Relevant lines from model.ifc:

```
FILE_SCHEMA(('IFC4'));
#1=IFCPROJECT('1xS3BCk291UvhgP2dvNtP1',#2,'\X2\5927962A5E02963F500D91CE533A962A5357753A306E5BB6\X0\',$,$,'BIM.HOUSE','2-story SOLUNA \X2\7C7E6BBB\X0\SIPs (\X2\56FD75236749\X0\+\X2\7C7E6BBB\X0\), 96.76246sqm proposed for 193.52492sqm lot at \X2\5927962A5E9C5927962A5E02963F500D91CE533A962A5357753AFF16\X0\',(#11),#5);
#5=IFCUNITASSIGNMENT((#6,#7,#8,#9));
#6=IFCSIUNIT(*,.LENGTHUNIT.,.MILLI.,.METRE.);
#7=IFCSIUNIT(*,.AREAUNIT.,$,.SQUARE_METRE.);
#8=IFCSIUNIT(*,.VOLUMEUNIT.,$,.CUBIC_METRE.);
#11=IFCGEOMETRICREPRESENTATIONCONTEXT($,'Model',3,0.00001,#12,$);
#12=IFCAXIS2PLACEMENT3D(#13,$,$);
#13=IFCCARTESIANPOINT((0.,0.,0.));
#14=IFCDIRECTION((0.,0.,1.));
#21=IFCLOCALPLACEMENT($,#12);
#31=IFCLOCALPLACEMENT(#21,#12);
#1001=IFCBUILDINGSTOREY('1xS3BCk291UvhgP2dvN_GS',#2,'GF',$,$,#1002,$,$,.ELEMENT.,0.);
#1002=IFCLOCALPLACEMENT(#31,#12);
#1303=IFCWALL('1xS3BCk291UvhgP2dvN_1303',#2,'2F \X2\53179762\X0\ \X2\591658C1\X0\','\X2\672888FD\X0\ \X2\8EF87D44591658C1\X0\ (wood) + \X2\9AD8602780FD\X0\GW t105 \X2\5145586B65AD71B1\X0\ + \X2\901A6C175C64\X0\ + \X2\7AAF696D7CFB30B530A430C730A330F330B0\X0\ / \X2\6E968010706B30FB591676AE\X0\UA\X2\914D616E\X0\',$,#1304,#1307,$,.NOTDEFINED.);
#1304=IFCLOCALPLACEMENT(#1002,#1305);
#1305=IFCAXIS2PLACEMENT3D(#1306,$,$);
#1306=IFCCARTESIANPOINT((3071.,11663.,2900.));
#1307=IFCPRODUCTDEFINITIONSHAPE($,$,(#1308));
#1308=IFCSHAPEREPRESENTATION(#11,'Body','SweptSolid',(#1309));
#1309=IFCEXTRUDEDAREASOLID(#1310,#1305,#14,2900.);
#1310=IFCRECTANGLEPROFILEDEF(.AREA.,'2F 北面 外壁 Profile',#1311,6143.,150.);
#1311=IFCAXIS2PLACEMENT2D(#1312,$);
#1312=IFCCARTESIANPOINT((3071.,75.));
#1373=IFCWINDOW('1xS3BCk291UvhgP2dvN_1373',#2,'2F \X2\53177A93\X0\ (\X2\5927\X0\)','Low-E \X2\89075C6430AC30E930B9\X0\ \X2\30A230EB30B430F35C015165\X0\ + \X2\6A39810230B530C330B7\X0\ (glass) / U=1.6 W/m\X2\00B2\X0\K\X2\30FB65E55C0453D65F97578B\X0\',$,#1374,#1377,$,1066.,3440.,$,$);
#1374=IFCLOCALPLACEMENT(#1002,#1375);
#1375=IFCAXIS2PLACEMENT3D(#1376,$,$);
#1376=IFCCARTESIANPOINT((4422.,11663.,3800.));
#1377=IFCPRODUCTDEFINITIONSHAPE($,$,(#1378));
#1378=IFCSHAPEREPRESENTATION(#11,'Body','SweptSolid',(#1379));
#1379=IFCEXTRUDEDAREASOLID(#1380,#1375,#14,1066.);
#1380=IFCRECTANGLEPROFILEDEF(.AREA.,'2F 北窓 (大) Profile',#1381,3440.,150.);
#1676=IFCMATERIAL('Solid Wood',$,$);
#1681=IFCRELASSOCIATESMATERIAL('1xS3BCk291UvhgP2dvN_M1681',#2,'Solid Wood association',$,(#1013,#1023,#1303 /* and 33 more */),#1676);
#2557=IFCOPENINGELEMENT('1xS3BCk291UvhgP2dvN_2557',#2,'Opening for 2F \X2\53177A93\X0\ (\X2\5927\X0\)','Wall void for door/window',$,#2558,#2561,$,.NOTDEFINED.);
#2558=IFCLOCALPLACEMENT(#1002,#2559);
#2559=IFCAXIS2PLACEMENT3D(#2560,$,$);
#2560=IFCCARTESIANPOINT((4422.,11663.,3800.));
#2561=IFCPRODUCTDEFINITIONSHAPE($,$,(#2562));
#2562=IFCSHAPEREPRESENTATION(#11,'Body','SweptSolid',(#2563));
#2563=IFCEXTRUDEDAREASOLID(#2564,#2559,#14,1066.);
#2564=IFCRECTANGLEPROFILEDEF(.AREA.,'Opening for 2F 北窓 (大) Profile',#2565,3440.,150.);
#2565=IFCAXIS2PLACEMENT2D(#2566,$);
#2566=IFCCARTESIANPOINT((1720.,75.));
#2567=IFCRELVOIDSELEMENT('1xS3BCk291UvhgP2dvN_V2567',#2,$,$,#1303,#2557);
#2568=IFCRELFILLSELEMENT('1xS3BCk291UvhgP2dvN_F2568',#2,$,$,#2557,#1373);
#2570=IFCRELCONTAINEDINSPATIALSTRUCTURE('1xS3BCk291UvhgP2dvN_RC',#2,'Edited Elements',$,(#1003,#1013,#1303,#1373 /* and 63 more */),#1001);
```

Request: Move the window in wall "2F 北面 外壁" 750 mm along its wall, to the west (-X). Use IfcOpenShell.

```python
import ifcopenshell
import ifcopenshell.api.geometry
import ifcopenshell.util.placement
import ifcopenshell.util.unit

model = ifcopenshell.open("model.ifc")
unit_scale = ifcopenshell.util.unit.calculate_unit_scale(model)

window = model.by_guid("1xS3BCk291UvhgP2dvN_1373")
opening = window.FillsVoids[0].RelatingOpeningElement
wall = opening.VoidsElements[0].RelatingBuildingElement

wall_matrix = ifcopenshell.util.placement.get_local_placement(wall.ObjectPlacement)
shift = wall_matrix[:3, 0] * -0.75 / unit_scale
before = ifcopenshell.util.placement.get_local_placement(window.ObjectPlacement)[:3, 3].copy()

# The window is not placed relative to its opening, so move both.
for product in (opening, window):
    matrix = ifcopenshell.util.placement.get_local_placement(product.ObjectPlacement)
    matrix[:3, 3] += shift
    ifcopenshell.api.geometry.edit_object_placement(model, product=product, matrix=matrix, is_si=False)

after = ifcopenshell.util.placement.get_local_placement(window.ObjectPlacement)[:3, 3]
print("window moved by", (after - before).round(3) + 0.0)

model.write("model_v2.ifc")
```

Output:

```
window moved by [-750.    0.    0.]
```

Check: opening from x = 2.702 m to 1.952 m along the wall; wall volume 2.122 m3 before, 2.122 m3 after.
